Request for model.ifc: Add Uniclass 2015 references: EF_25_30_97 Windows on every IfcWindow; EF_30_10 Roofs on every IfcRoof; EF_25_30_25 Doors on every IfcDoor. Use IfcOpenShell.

First a look at what the model holds.

```python
import ifcopenshell

model = ifcopenshell.open("model.ifc")
print(model.schema)
print("classifications:", [c.Name for c in model.by_type("IfcClassification")])
for ifc_class in ("IfcDoor", "IfcRoof", "IfcStair", "IfcWall", "IfcWindow"):
    print(ifc_class, len(model.by_type(ifc_class)))
```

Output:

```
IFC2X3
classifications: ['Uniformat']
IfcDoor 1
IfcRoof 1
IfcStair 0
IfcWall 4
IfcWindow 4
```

```python
import ifcopenshell
import ifcopenshell.api.classification

model = ifcopenshell.open("model.ifc")

# IFC2X3 requires Source and Edition and has no link from the project to the system.
system = model.create_entity("IfcClassification", Source="NBS", Edition="2015", Name="Uniclass 2015")

codes = {
    "IfcWindow": ("EF_25_30_97", "Windows"),
    "IfcRoof": ("EF_30_10", "Roofs"),
    "IfcDoor": ("EF_25_30_25", "Doors"),
}
for ifc_class, (code, name) in codes.items():
    products = model.by_type(ifc_class)
    ifcopenshell.api.classification.add_reference(
        model, products=products, classification=system, identification=code, name=name
    )
    print(code, len(products))

model.write("model_v2.ifc")
```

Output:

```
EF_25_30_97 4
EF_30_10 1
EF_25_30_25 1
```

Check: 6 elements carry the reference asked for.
